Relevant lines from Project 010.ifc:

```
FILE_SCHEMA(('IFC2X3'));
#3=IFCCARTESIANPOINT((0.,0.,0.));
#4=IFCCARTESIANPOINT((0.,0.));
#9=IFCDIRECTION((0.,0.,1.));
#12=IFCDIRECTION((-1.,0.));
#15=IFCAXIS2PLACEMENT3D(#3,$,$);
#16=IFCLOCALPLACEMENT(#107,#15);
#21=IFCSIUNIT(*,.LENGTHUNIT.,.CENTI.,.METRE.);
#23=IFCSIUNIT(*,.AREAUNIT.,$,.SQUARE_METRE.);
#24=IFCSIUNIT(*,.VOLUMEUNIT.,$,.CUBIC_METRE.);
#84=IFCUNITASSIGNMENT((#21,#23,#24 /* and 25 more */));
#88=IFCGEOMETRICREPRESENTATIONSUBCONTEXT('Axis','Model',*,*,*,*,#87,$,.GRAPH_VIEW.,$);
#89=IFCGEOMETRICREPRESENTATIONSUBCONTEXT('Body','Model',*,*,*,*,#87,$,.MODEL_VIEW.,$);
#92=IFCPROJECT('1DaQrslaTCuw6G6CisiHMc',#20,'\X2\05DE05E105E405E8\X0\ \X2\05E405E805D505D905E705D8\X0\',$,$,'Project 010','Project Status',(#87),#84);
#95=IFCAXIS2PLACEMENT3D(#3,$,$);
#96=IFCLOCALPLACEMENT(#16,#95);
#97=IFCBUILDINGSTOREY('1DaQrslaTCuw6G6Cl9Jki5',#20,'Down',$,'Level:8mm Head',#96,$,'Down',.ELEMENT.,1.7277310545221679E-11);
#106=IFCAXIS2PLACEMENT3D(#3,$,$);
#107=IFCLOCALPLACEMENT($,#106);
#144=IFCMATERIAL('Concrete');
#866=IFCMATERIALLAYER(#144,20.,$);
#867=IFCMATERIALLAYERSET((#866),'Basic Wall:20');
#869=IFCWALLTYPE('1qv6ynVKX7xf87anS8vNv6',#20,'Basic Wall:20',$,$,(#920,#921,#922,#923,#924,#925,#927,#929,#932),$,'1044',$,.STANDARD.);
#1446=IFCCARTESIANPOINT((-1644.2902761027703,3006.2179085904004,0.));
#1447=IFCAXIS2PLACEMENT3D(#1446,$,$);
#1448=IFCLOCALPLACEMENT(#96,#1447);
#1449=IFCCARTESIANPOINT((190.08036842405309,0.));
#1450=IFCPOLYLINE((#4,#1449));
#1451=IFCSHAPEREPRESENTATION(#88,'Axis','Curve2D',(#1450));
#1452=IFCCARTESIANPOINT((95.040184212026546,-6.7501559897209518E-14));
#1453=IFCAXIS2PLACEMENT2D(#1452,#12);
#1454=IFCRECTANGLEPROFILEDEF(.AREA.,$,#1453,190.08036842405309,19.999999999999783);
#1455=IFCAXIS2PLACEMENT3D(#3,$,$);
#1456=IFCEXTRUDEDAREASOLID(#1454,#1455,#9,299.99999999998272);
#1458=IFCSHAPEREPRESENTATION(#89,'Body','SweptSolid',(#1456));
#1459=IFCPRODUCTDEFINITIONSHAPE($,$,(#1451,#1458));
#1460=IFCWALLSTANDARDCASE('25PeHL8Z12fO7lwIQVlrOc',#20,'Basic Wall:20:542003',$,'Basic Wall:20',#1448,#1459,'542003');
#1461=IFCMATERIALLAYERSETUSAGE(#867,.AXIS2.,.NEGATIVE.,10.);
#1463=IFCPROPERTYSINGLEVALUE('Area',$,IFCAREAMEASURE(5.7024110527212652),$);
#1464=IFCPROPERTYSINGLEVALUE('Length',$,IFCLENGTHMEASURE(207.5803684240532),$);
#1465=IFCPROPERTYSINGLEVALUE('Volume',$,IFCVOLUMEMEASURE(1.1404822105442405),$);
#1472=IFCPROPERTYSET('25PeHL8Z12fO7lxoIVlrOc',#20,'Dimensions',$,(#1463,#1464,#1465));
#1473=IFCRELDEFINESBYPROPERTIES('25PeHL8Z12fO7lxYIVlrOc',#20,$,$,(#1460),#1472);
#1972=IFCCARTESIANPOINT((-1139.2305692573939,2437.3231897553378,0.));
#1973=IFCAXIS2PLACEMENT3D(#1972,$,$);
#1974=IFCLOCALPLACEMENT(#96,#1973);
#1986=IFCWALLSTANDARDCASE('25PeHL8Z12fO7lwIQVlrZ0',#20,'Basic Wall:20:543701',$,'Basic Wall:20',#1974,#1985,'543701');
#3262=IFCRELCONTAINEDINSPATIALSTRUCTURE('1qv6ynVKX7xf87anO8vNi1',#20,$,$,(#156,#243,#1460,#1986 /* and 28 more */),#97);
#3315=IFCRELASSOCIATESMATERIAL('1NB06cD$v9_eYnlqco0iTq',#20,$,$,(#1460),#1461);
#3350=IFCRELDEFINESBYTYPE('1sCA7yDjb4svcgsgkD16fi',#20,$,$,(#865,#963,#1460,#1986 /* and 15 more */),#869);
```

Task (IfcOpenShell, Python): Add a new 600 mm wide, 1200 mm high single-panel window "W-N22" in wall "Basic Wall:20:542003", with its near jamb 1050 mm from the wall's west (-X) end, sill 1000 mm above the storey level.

```python
import numpy as np
import ifcopenshell
import ifcopenshell.api.feature
import ifcopenshell.api.geometry
import ifcopenshell.api.pset
import ifcopenshell.api.root
import ifcopenshell.api.spatial
import ifcopenshell.api.type
import ifcopenshell.geom
import ifcopenshell.util.element
import ifcopenshell.util.placement
import ifcopenshell.util.representation
import ifcopenshell.util.shape
import ifcopenshell.util.unit

model = ifcopenshell.open("Project 010.ifc")
unit_scale = ifcopenshell.util.unit.calculate_unit_scale(model)
area_scale = ifcopenshell.util.unit.calculate_unit_scale(model, "AREAUNIT")
volume_scale = ifcopenshell.util.unit.calculate_unit_scale(model, "VOLUMEUNIT")
settings = ifcopenshell.geom.settings()


def volume(element):
    """Net volume in cubic metres, openings subtracted."""
    shape = ifcopenshell.geom.create_shape(settings, element)
    return ifcopenshell.util.shape.get_volume(shape.geometry)


wall = model.by_guid("25PeHL8Z12fO7lwIQVlrOc")
storey = ifcopenshell.util.element.get_container(wall, ifc_class="IfcBuildingStorey")
context = ifcopenshell.util.representation.get_context(model, "Model", "Body", "MODEL_VIEW")
before = volume(wall)

width, height, from_end, sill = 0.6, 1.2, 1.05, 1  # metres

# The wall runs along its own X axis, and the end named is its -X end.
wall_shape = ifcopenshell.geom.create_shape(settings, wall)
x, y, z = ifcopenshell.util.shape.get_vertices(wall_shape.geometry).T
start = x.min() + from_end
face, thickness = float(y.min()), float(y.max() - y.min())
wall_matrix = ifcopenshell.util.placement.get_local_placement(wall.ObjectPlacement)
level = ifcopenshell.util.placement.get_local_placement(storey.ObjectPlacement)[2, 3]


def in_wall(x, y):
    """Placement at x, y metres in the wall's axes, at sill height."""
    matrix = wall_matrix.copy()
    matrix[:, 3] = wall_matrix @ np.array([x / unit_scale, y / unit_scale, 0.0, 1.0])
    matrix[2, 3] = level + sill / unit_scale
    return matrix


# Opening: a box that overshoots both wall faces by 50 mm.
opening = ifcopenshell.api.root.create_entity(model, ifc_class="IfcOpeningElement")
box = ifcopenshell.api.geometry.add_wall_representation(
    model, context=context, length=width, height=height, thickness=thickness + 0.1
)
ifcopenshell.api.geometry.assign_representation(model, product=opening, representation=box)
ifcopenshell.api.geometry.edit_object_placement(model, product=opening, matrix=in_wall(start, face - 0.05), is_si=False)
ifcopenshell.api.feature.add_feature(model, feature=opening, element=wall)

window = ifcopenshell.api.root.create_entity(model, ifc_class="IfcWindow", name="W-N22")
window.OverallWidth, window.OverallHeight = width / unit_scale, height / unit_scale
body = ifcopenshell.api.geometry.add_window_representation(
    model,
    context=context,
    overall_width=window.OverallWidth,
    overall_height=window.OverallHeight,
    partition_type="SINGLE_PANEL",
)
ifcopenshell.api.geometry.assign_representation(model, product=window, representation=body)
ifcopenshell.api.spatial.assign_container(model, products=[window], relating_structure=storey)
fills = ifcopenshell.api.feature.add_filling(model, opening=opening, element=window)
fills.OwnerHistory = window.OwnerHistory  # required in IFC2X3

# IFC2X3 keeps the operation on the window style.
style = ifcopenshell.api.root.create_entity(model, ifc_class="IfcWindowStyle", name="W-N22")
style.OperationType, style.ConstructionType = "SINGLE_PANEL", "NOTDEFINED"
style.ParameterTakesPrecedence = style.Sizeable = False
ifcopenshell.api.type.assign_type(model, related_objects=[window], relating_type=style)

# Centre the window in the wall's thickness.
ifcopenshell.api.geometry.edit_object_placement(model, product=window, matrix=in_wall(start, face), is_si=False)
window_shape = ifcopenshell.geom.create_shape(settings, window)
depth = ifcopenshell.util.shape.get_vertices(window_shape.geometry)[:, 1]
offset = face + thickness / 2 - (depth.min() + depth.max()) / 2
ifcopenshell.api.geometry.edit_object_placement(model, product=window, matrix=in_wall(start, offset), is_si=False)

after = volume(wall)

# Update the wall's stored quantities.
pset = model.by_id(ifcopenshell.util.element.get_pset(wall, "Dimensions", should_inherit=False)["id"])
ifcopenshell.api.pset.edit_pset(model, pset=pset, properties={
    "Area": model.create_entity("IfcAreaMeasure", after / thickness / area_scale),
    "Volume": model.create_entity("IfcVolumeMeasure", after / volume_scale),
})

print(f"wall volume {before:.3f} -> {after:.3f} m3")

model.write("Project 010_v2.ifc")
```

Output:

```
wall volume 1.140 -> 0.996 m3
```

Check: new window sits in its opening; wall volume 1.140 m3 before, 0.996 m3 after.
